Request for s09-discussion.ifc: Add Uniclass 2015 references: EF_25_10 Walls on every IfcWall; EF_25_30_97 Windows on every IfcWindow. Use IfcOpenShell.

First a look at what the model holds.

```python
import ifcopenshell

model = ifcopenshell.open("s09-discussion.ifc")
print(model.schema)
print("classifications:", [c.Name for c in model.by_type("IfcClassification")])
for ifc_class in ("IfcDoor", "IfcRoof", "IfcStair", "IfcWall", "IfcWindow"):
    print(ifc_class, len(model.by_type(ifc_class)))
```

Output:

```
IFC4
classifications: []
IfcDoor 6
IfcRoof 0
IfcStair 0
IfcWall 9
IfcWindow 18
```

```python
import ifcopenshell
import ifcopenshell.api.classification

model = ifcopenshell.open("s09-discussion.ifc")

system = ifcopenshell.api.classification.add_classification(model, classification="Uniclass 2015")

codes = {
    "IfcWall": ("EF_25_10", "Walls"),
    "IfcWindow": ("EF_25_30_97", "Windows"),
}
for ifc_class, (code, name) in codes.items():
    products = model.by_type(ifc_class)
    ifcopenshell.api.classification.add_reference(
        model, products=products, classification=system, identification=code, name=name
    )
    print(code, len(products))

model.write("s09-discussion_rev.ifc")
```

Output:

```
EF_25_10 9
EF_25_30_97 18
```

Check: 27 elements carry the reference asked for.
